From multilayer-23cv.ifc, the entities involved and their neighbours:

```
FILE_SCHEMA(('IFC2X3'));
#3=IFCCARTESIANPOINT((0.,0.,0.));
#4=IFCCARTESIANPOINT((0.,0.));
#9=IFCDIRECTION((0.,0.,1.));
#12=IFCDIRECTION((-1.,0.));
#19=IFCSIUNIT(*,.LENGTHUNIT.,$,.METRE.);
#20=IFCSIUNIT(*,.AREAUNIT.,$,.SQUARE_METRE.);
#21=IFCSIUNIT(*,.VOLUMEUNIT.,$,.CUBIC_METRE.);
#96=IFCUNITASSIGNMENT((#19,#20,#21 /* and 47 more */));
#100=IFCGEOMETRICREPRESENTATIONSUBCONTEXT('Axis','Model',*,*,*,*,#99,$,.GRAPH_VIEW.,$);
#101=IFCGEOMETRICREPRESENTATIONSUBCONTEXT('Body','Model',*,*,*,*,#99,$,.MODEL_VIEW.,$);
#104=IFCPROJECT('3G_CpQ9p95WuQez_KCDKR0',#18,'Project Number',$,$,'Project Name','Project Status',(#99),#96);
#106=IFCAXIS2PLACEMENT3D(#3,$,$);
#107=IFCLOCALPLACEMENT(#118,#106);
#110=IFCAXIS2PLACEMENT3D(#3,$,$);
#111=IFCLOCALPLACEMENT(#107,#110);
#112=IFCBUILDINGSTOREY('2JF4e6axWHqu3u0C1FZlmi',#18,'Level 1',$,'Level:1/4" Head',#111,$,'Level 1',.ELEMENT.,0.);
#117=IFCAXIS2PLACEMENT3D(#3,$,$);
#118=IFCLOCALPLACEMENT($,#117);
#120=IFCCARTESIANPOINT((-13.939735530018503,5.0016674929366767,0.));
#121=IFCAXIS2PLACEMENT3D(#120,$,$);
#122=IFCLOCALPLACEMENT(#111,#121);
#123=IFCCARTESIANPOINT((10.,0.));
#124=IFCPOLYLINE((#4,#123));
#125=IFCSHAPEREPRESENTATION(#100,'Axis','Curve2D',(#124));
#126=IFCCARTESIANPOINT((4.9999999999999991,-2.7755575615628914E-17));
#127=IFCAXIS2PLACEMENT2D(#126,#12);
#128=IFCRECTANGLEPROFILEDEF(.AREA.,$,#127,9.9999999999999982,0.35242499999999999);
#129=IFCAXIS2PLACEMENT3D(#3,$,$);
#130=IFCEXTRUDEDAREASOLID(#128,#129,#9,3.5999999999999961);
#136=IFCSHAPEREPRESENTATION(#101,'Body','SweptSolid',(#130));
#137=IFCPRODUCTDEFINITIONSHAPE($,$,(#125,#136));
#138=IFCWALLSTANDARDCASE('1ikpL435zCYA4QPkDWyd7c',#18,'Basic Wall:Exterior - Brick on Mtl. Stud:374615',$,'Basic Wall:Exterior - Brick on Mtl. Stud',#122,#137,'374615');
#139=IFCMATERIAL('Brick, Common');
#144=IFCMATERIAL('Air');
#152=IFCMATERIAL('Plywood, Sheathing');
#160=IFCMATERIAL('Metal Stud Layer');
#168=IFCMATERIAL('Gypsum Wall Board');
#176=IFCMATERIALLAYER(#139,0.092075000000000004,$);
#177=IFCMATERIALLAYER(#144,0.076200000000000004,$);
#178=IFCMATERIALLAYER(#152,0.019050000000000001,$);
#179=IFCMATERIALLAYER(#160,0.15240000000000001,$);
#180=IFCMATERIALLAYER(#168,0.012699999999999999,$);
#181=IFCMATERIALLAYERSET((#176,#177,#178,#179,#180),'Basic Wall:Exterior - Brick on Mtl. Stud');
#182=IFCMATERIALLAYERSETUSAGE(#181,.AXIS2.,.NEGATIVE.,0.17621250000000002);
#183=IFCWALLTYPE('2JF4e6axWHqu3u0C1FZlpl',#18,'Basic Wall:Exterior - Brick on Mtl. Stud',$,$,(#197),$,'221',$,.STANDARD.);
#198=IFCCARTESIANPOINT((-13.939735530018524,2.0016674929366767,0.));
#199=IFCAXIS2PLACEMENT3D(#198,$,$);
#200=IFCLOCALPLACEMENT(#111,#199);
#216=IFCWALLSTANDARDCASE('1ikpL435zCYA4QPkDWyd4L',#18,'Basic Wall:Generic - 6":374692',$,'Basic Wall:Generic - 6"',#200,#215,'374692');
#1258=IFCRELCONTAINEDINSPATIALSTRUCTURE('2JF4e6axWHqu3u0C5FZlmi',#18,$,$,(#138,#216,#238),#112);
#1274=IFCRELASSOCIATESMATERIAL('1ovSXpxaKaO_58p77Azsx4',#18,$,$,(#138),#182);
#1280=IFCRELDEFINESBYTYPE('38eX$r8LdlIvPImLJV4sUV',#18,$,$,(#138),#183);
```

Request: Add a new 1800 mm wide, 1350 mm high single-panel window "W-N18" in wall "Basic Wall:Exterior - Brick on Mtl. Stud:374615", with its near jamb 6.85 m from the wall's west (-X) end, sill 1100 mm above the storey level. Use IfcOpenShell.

```python
import numpy as np
import ifcopenshell
import ifcopenshell.api.feature
import ifcopenshell.api.geometry
import ifcopenshell.api.root
import ifcopenshell.api.spatial
import ifcopenshell.api.type
import ifcopenshell.geom
import ifcopenshell.util.element
import ifcopenshell.util.placement
import ifcopenshell.util.representation
import ifcopenshell.util.shape
import ifcopenshell.util.unit

model = ifcopenshell.open("multilayer-23cv.ifc")
unit_scale = ifcopenshell.util.unit.calculate_unit_scale(model)
settings = ifcopenshell.geom.settings()


def volume(element):
    """Net volume in cubic metres, openings subtracted."""
    shape = ifcopenshell.geom.create_shape(settings, element)
    return ifcopenshell.util.shape.get_volume(shape.geometry)


wall = model.by_id(138)
storey = ifcopenshell.util.element.get_container(wall, ifc_class="IfcBuildingStorey")
context = ifcopenshell.util.representation.get_context(model, "Model", "Body", "MODEL_VIEW")
before = volume(wall)

width, height, from_end, sill = 1.8, 1.35, 6.85, 1.1  # metres

# The wall runs along its own X axis, and the end named is its -X end.
wall_shape = ifcopenshell.geom.create_shape(settings, wall)
x, y, z = ifcopenshell.util.shape.get_vertices(wall_shape.geometry).T
start = x.min() + from_end
face, thickness = float(y.min()), float(y.max() - y.min())
wall_matrix = ifcopenshell.util.placement.get_local_placement(wall.ObjectPlacement)
level = ifcopenshell.util.placement.get_local_placement(storey.ObjectPlacement)[2, 3]


def in_wall(x, y):
    """Placement at x, y metres in the wall's axes, at sill height."""
    matrix = wall_matrix.copy()
    matrix[:, 3] = wall_matrix @ np.array([x / unit_scale, y / unit_scale, 0.0, 1.0])
    matrix[2, 3] = level + sill / unit_scale
    return matrix


# Opening: a box that overshoots both wall faces by 50 mm.
opening = ifcopenshell.api.root.create_entity(model, ifc_class="IfcOpeningElement")
box = ifcopenshell.api.geometry.add_wall_representation(
    model, context=context, length=width, height=height, thickness=thickness + 0.1
)
ifcopenshell.api.geometry.assign_representation(model, product=opening, representation=box)
ifcopenshell.api.geometry.edit_object_placement(model, product=opening, matrix=in_wall(start, face - 0.05), is_si=False)
ifcopenshell.api.feature.add_feature(model, feature=opening, element=wall)

window = ifcopenshell.api.root.create_entity(model, ifc_class="IfcWindow", name="W-N18")
window.OverallWidth, window.OverallHeight = width / unit_scale, height / unit_scale
body = ifcopenshell.api.geometry.add_window_representation(
    model,
    context=context,
    overall_width=window.OverallWidth,
    overall_height=window.OverallHeight,
    partition_type="SINGLE_PANEL",
)
ifcopenshell.api.geometry.assign_representation(model, product=window, representation=body)
ifcopenshell.api.spatial.assign_container(model, products=[window], relating_structure=storey)
fills = ifcopenshell.api.feature.add_filling(model, opening=opening, element=window)
fills.OwnerHistory = window.OwnerHistory  # required in IFC2X3

# IFC2X3 keeps the operation on the window style.
style = ifcopenshell.api.root.create_entity(model, ifc_class="IfcWindowStyle", name="W-N18")
style.OperationType, style.ConstructionType = "SINGLE_PANEL", "NOTDEFINED"
style.ParameterTakesPrecedence = style.Sizeable = False
ifcopenshell.api.type.assign_type(model, related_objects=[window], relating_type=style)

# Centre the window in the wall's thickness.
ifcopenshell.api.geometry.edit_object_placement(model, product=window, matrix=in_wall(start, face), is_si=False)
window_shape = ifcopenshell.geom.create_shape(settings, window)
depth = ifcopenshell.util.shape.get_vertices(window_shape.geometry)[:, 1]
offset = face + thickness / 2 - (depth.min() + depth.max()) / 2
ifcopenshell.api.geometry.edit_object_placement(model, product=window, matrix=in_wall(start, offset), is_si=False)

after = volume(wall)

print(f"wall volume {before:.3f} -> {after:.3f} m3")

model.write("multilayer-23cv_rev.ifc")
```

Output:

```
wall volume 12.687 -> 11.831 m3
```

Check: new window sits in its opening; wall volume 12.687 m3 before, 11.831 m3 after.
